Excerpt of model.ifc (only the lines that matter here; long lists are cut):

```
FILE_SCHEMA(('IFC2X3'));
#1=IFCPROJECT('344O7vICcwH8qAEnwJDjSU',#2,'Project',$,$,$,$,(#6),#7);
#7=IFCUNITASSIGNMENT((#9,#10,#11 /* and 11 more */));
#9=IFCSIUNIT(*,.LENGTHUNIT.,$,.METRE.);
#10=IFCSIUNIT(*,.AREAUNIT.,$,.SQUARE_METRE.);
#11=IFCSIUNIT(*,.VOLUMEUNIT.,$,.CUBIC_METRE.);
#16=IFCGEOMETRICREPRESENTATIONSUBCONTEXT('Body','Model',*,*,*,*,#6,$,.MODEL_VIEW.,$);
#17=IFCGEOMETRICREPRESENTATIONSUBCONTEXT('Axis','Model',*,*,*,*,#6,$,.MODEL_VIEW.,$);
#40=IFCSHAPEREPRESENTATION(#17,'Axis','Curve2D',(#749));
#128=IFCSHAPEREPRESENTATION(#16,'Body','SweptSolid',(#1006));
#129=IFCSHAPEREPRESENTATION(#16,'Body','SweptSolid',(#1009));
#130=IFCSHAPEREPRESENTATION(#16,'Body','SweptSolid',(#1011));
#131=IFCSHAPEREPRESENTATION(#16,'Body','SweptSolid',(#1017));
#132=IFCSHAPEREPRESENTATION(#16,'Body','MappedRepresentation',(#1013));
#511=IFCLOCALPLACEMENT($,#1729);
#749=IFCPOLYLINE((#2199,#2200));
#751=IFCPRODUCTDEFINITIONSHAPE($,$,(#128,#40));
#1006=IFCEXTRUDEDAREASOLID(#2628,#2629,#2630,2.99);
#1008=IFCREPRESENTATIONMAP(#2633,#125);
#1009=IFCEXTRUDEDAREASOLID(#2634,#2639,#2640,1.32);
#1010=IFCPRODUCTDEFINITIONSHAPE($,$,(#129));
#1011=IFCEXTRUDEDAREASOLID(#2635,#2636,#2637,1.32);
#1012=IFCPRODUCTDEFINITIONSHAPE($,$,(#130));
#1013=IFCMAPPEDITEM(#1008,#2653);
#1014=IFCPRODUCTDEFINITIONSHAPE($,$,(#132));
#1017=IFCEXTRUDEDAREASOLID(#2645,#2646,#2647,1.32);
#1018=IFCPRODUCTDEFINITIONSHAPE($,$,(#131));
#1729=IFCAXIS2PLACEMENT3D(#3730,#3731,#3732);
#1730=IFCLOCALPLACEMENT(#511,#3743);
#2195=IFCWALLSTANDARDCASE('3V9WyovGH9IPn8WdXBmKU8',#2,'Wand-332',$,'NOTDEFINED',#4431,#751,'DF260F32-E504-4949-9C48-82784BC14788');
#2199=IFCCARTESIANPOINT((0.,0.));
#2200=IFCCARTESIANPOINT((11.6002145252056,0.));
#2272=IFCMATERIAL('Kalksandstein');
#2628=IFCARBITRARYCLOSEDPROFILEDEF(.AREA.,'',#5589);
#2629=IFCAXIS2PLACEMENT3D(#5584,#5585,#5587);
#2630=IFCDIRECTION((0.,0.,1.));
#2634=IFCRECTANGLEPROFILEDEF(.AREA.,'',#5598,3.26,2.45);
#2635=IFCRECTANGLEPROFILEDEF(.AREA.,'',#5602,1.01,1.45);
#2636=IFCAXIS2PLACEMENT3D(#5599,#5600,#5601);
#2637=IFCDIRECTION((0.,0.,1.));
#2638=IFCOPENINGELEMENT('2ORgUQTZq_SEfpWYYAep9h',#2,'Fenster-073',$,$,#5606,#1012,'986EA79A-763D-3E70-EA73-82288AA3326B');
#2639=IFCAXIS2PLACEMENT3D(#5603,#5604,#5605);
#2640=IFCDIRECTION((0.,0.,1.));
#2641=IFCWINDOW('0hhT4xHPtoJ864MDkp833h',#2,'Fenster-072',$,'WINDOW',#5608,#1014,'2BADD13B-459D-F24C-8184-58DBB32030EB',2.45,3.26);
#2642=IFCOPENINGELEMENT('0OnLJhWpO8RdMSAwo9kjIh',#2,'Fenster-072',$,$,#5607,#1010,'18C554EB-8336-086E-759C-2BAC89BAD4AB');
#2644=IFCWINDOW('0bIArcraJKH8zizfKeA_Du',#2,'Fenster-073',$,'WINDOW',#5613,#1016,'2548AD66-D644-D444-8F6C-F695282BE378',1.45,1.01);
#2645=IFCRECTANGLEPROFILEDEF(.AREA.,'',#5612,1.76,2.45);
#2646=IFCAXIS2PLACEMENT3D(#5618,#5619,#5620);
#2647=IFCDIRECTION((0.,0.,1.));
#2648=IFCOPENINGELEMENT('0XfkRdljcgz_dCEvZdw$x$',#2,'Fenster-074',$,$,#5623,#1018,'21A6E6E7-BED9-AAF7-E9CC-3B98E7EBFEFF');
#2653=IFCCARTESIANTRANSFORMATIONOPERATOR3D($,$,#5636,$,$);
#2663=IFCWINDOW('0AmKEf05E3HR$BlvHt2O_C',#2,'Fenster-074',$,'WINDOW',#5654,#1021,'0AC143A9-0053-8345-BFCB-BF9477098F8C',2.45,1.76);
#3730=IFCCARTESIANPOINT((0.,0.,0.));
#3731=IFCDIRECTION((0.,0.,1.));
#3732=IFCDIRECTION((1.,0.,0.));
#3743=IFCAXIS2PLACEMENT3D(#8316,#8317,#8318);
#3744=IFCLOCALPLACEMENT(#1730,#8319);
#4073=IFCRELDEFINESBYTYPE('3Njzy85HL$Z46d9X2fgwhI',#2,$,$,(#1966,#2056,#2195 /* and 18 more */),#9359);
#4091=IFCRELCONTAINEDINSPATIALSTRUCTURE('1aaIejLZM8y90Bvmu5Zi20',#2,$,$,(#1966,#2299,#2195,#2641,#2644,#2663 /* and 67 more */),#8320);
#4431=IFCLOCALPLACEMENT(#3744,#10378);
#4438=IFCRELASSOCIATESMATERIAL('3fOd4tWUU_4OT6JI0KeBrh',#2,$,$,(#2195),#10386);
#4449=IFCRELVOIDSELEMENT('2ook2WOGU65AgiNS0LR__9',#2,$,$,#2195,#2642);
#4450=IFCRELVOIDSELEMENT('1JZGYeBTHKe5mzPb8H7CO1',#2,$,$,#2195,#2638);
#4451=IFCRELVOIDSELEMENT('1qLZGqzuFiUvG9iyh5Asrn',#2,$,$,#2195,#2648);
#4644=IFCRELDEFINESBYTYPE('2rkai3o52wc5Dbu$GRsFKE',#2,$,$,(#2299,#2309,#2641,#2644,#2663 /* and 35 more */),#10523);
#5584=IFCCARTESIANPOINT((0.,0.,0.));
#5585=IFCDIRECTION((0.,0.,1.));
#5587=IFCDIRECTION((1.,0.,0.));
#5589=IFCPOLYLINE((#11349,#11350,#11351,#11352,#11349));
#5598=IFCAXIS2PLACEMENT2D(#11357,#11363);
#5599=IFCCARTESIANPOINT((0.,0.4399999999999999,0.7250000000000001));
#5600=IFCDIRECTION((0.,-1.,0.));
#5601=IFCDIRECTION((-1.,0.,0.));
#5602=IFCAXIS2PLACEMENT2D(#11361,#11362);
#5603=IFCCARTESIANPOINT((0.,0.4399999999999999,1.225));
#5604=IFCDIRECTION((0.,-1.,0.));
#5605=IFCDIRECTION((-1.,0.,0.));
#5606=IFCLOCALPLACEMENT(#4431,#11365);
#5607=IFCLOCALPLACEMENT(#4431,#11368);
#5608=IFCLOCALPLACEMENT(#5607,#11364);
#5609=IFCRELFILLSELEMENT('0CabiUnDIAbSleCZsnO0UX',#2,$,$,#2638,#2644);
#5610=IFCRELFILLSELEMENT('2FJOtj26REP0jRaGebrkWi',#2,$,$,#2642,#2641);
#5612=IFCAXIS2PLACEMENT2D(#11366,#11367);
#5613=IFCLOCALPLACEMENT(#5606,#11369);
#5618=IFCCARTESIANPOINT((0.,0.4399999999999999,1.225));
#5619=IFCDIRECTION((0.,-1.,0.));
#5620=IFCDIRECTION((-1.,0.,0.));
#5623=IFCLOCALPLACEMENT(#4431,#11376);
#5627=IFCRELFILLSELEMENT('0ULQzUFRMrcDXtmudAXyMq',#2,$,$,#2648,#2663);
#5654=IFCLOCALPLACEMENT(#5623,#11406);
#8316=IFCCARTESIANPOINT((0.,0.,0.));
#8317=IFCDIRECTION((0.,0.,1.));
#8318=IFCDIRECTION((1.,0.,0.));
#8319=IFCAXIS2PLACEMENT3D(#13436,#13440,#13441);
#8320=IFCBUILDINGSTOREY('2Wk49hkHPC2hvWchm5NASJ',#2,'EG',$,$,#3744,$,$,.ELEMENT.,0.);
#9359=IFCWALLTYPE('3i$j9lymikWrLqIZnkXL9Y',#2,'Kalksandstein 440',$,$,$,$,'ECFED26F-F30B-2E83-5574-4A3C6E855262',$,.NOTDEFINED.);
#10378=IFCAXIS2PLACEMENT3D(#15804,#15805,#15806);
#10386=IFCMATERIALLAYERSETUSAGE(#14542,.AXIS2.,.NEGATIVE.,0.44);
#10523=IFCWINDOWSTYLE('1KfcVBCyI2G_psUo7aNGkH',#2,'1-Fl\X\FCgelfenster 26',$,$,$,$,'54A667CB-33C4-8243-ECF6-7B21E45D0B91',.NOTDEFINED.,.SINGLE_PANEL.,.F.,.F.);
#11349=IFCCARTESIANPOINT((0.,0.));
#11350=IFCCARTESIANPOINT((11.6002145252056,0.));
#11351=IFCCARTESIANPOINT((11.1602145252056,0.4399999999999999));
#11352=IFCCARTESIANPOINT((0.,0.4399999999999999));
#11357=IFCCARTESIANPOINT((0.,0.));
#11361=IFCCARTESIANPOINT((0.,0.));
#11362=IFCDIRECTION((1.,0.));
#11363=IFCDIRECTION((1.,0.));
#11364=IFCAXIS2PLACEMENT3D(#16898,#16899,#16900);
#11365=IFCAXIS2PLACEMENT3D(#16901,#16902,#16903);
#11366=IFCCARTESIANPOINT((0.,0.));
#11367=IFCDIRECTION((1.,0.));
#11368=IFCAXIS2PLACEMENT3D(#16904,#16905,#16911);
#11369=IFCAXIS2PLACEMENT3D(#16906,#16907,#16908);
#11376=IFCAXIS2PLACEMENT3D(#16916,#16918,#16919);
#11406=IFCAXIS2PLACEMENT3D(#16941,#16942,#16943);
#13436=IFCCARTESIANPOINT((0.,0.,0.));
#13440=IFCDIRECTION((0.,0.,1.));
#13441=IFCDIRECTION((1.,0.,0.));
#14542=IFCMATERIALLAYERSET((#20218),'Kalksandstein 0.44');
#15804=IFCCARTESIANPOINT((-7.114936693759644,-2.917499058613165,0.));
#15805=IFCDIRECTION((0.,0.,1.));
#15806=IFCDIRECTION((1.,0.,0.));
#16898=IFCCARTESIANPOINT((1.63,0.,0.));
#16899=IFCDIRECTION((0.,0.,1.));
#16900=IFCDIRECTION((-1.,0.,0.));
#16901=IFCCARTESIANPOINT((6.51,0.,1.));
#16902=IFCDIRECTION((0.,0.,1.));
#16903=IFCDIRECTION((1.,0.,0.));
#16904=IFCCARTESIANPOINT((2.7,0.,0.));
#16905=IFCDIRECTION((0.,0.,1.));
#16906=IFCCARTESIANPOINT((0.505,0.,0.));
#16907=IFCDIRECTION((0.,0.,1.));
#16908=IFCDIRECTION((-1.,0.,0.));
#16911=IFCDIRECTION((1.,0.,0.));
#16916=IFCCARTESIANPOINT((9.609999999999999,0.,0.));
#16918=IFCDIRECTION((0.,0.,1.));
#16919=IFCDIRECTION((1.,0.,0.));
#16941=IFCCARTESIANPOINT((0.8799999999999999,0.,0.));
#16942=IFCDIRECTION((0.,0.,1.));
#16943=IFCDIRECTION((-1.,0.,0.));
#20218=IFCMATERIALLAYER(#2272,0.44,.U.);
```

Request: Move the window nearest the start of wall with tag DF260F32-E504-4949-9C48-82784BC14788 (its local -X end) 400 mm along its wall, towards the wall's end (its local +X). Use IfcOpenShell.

```python
import ifcopenshell
import ifcopenshell.api.geometry
import ifcopenshell.util.placement

model = ifcopenshell.open("model.ifc")

window = model.by_guid("0hhT4xHPtoJ864MDkp833h")
opening = window.FillsVoids[0].RelatingOpeningElement
wall = opening.VoidsElements[0].RelatingBuildingElement

wall_matrix = ifcopenshell.util.placement.get_local_placement(wall.ObjectPlacement)
shift = wall_matrix[:3, 0] * 0.4
before = ifcopenshell.util.placement.get_local_placement(window.ObjectPlacement)[:3, 3].copy()

# The window is placed relative to its opening, so it follows when the opening moves.
matrix = ifcopenshell.util.placement.get_local_placement(opening.ObjectPlacement)
matrix[:3, 3] += shift
ifcopenshell.api.geometry.edit_object_placement(
    model, product=opening, matrix=matrix, is_si=False, should_transform_children=True
)

after = ifcopenshell.util.placement.get_local_placement(window.ObjectPlacement)[:3, 3]
print("window moved by", (after - before).round(3) + 0.0)

model.write("model_rev.ifc")
```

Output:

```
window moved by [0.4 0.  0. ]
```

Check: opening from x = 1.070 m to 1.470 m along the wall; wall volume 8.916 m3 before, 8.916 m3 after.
